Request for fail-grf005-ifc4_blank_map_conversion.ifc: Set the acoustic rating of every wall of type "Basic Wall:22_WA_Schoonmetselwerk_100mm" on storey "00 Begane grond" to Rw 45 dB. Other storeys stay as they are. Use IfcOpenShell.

First a look at what the model holds.

```python
import ifcopenshell
import ifcopenshell.util.element

model = ifcopenshell.open("fail-grf005-ifc4_blank_map_conversion.ifc")
print(model.schema)
storey = next(s for s in model.by_type("IfcBuildingStorey") if s.Name == "00 Begane grond")
walls = [e for e in ifcopenshell.util.element.get_decomposition(storey) if e.is_a("IfcWall")]
seen = {}
for e in walls:
    element_type = ifcopenshell.util.element.get_type(e)
    key = (element_type.Name if element_type != e and element_type else None, ifcopenshell.util.element.get_pset(e, "Pset_WallCommon", "AcousticRating"))
    seen[key] = seen.get(key, 0) + 1
for (name, value), count in sorted(seen.items(), key=str):
    print(count, "x", name, "|", value)
```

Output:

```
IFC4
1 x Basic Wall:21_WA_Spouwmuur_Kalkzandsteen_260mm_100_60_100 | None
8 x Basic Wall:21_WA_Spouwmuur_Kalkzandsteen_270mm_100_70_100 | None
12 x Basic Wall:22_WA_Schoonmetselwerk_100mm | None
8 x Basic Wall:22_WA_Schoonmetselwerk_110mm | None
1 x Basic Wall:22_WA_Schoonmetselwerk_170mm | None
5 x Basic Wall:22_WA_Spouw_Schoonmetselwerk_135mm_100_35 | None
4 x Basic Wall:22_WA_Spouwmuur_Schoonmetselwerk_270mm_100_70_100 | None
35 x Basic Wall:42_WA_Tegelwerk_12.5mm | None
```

```python
import ifcopenshell
import ifcopenshell.api.pset
import ifcopenshell.util.element

model = ifcopenshell.open("fail-grf005-ifc4_blank_map_conversion.ifc")

storey = next(s for s in model.by_type("IfcBuildingStorey") if s.Name == "00 Begane grond")
walls = [e for e in ifcopenshell.util.element.get_decomposition(storey) if e.is_a("IfcWall")]

count = 0
for e in walls:
    element_type = ifcopenshell.util.element.get_type(e)
    if element_type in (None, e) or element_type.Name != "Basic Wall:22_WA_Schoonmetselwerk_100mm":
        continue
    # add_pset returns the element's existing set when there is one.
    pset = ifcopenshell.api.pset.add_pset(model, product=e, name="Pset_WallCommon")
    ifcopenshell.api.pset.edit_pset(model, pset=pset, properties={"AcousticRating": "Rw 45 dB"})
    count += 1

print(count, "walls updated")

model.write("fail-grf005-ifc4_blank_map_conversion_updated.ifc")
```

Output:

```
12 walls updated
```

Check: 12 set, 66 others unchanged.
